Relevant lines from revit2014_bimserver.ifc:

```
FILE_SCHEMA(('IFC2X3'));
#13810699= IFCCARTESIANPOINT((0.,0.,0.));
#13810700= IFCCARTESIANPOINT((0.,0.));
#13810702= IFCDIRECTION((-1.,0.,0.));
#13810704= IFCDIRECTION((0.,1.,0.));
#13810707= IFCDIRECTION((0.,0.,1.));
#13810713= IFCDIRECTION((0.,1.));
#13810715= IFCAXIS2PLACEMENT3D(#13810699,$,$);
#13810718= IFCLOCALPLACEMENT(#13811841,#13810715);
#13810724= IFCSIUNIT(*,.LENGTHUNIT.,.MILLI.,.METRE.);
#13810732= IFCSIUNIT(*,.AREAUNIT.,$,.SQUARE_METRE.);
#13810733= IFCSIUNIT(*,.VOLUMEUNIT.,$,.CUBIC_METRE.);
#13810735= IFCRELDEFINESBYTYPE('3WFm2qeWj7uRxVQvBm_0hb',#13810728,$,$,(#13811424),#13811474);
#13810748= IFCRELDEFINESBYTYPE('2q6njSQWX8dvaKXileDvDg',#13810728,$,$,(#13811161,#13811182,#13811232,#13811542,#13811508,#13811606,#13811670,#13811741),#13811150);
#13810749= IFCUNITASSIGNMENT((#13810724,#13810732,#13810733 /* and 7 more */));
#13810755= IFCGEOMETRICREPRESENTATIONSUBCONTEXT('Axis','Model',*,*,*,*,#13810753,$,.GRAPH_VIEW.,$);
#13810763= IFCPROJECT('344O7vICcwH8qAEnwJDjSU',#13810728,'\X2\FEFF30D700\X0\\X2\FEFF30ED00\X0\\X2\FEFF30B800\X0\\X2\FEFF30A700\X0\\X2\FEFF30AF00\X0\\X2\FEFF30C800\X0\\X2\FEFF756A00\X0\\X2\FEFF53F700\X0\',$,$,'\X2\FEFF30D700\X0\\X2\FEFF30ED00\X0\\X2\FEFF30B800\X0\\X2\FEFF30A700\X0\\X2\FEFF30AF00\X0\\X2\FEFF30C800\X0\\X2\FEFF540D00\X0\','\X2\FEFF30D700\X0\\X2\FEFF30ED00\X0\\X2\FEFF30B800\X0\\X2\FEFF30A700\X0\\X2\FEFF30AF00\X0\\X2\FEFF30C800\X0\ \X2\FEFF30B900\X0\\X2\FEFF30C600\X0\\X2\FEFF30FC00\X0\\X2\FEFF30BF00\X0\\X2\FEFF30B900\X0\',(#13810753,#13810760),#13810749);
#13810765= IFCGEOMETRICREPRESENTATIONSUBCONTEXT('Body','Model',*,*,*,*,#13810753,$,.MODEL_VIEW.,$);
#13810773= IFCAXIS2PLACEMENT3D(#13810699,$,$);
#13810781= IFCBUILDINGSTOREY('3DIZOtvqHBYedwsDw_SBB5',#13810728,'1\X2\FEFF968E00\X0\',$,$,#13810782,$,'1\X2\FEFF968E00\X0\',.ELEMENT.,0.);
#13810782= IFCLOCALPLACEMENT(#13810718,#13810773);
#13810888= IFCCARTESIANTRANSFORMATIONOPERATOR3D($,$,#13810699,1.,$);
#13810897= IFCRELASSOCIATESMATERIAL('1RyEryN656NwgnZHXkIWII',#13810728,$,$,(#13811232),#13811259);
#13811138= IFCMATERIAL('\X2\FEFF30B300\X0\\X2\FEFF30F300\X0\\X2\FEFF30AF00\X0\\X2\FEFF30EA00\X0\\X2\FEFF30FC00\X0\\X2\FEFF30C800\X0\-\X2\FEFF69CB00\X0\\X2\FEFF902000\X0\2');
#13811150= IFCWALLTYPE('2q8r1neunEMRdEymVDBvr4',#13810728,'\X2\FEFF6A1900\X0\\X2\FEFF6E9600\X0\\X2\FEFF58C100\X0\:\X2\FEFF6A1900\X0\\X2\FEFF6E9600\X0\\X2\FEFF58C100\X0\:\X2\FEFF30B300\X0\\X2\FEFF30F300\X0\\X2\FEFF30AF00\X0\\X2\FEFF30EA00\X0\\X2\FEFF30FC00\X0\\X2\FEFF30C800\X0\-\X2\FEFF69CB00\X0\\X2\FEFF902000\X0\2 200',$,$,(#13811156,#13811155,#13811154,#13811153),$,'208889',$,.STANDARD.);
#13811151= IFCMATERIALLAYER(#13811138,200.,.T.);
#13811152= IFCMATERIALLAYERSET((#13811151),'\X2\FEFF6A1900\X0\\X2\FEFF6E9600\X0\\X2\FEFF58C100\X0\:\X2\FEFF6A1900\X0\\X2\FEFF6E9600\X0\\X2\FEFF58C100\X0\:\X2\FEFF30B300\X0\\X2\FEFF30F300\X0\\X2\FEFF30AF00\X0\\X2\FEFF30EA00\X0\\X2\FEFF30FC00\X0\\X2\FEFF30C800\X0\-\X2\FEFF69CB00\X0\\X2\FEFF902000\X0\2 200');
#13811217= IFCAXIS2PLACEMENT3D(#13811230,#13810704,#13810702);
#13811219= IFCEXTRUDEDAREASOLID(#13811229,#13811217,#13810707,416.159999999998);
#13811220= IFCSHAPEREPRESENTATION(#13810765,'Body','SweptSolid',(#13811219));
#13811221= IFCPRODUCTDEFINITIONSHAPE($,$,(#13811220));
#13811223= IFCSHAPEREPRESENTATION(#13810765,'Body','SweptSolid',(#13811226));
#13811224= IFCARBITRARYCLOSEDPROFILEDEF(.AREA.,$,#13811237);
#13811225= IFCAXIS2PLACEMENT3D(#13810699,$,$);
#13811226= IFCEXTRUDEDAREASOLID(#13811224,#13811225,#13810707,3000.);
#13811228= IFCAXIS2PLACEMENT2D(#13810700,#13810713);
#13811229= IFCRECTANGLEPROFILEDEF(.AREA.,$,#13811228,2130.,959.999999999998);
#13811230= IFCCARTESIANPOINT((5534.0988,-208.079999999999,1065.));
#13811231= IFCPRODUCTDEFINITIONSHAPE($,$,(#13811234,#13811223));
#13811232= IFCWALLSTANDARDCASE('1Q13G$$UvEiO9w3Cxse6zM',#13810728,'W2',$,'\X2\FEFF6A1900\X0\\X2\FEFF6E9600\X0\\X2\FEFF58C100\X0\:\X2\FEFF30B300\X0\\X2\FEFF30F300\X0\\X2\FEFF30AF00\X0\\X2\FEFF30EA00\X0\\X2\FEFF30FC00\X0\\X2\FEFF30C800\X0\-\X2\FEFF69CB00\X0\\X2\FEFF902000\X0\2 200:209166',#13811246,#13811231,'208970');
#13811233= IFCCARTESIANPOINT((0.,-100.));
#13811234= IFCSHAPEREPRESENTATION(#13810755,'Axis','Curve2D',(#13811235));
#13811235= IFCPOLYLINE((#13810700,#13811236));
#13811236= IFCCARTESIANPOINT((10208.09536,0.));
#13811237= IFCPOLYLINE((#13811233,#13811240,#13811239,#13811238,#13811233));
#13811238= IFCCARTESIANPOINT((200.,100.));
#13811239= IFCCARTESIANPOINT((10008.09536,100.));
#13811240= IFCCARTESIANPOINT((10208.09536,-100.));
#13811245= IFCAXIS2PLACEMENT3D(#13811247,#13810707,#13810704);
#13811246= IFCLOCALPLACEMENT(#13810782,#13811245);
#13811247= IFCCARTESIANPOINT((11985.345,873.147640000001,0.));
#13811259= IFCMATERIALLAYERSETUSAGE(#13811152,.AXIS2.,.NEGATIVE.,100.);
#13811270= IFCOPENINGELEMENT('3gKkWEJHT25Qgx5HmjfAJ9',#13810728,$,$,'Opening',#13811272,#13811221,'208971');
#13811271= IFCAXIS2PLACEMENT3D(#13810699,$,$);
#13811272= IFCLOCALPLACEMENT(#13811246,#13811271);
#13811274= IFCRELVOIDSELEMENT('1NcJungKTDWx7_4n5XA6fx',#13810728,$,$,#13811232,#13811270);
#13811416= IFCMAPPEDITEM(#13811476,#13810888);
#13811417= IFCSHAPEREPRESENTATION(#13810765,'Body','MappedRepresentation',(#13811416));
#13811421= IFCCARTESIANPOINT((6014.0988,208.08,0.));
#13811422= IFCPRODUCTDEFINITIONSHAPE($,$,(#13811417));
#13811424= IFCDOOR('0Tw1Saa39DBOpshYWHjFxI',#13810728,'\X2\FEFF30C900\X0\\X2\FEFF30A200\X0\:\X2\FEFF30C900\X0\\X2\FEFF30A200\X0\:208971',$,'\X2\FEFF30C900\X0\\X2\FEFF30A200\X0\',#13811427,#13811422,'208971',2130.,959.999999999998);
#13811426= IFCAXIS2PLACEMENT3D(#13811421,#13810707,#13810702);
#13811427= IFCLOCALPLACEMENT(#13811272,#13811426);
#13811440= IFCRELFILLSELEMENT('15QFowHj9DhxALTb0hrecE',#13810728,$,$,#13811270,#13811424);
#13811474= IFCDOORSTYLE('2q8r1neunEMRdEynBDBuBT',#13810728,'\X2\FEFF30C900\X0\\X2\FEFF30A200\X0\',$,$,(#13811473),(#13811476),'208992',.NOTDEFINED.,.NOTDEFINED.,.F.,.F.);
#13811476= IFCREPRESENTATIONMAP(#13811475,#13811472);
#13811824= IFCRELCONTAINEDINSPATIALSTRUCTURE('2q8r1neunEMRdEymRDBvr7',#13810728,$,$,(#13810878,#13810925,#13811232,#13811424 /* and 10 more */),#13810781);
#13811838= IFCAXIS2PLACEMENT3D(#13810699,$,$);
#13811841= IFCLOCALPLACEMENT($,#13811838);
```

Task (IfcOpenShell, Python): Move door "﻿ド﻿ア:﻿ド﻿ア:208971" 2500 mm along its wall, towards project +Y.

```python
import ifcopenshell
import ifcopenshell.api.geometry
import ifcopenshell.util.placement

model = ifcopenshell.open("revit2014_bimserver.ifc")

door = model.by_guid("0Tw1Saa39DBOpshYWHjFxI")
opening = door.FillsVoids[0].RelatingOpeningElement
wall = opening.VoidsElements[0].RelatingBuildingElement

wall_matrix = ifcopenshell.util.placement.get_local_placement(wall.ObjectPlacement)
shift = wall_matrix[:3, 0] * 2500.0
before = ifcopenshell.util.placement.get_local_placement(door.ObjectPlacement)[:3, 3].copy()

# The door is placed relative to its opening, so it follows when the opening moves.
matrix = ifcopenshell.util.placement.get_local_placement(opening.ObjectPlacement)
matrix[:3, 3] += shift
ifcopenshell.api.geometry.edit_object_placement(
    model, product=opening, matrix=matrix, is_si=False, should_transform_children=True
)

after = ifcopenshell.util.placement.get_local_placement(door.ObjectPlacement)[:3, 3]
print("door moved by", (after - before).round(3) + 0.0)

model.write("revit2014_bimserver_v2.ifc")
```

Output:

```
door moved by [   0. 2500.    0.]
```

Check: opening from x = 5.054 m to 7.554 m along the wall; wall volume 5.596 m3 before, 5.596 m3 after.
